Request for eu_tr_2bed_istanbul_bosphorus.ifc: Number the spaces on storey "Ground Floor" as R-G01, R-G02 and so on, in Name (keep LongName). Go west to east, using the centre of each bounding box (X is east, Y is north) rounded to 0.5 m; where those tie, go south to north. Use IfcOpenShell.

First a look at what the model holds.

```python
import ifcopenshell
import ifcopenshell.util.element
import ifcopenshell.util.placement

model = ifcopenshell.open("eu_tr_2bed_istanbul_bosphorus.ifc")
print(model.schema)
storey = next(s for s in model.by_type("IfcBuildingStorey") if s.Name == "Ground Floor")
spaces = [e for e in ifcopenshell.util.element.get_decomposition(storey) if e.is_a("IfcSpace")]
for e in sorted(spaces, key=lambda e: e.id()):
    origin = ifcopenshell.util.placement.get_local_placement(e.ObjectPlacement)[:3, 3]
    print(e.id(), e.Name, e.LongName, origin.round(2) + 0.0, sep=" | ")
```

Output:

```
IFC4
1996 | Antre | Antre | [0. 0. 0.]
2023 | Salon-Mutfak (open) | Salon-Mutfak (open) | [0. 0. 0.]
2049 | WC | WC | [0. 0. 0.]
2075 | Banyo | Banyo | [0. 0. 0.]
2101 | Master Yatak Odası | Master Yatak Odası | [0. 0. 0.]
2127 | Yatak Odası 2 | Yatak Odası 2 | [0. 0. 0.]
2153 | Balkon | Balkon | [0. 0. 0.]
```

```python
import ifcopenshell
import ifcopenshell.geom
import ifcopenshell.util.element
import ifcopenshell.util.shape

model = ifcopenshell.open("eu_tr_2bed_istanbul_bosphorus.ifc")
settings = ifcopenshell.geom.settings()
settings.set("use-world-coords", True)


def centre(element):
    shape = ifcopenshell.geom.create_shape(settings, element)
    return ifcopenshell.util.shape.get_bbox_centroid(shape.geometry)


storey = next(s for s in model.by_type("IfcBuildingStorey") if s.Name == "Ground Floor")
spaces = [e for e in ifcopenshell.util.element.get_decomposition(storey) if e.is_a("IfcSpace")]

# Insertion points can sit at a corner or the storey origin, so sort by the geometry (in metres).
centres = {e: centre(e) for e in spaces}
spaces.sort(key=lambda e: (round(centres[e][0] / 0.5), centres[e][1]))

for i, e in enumerate(spaces, start=1):
    number = f"R-G{i:02d}"
    e.Name = number
    print(e.id(), number)

model.write("eu_tr_2bed_istanbul_bosphorus-out.ifc")
```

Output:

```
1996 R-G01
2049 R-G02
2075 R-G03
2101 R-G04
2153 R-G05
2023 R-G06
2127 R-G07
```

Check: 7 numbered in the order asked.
